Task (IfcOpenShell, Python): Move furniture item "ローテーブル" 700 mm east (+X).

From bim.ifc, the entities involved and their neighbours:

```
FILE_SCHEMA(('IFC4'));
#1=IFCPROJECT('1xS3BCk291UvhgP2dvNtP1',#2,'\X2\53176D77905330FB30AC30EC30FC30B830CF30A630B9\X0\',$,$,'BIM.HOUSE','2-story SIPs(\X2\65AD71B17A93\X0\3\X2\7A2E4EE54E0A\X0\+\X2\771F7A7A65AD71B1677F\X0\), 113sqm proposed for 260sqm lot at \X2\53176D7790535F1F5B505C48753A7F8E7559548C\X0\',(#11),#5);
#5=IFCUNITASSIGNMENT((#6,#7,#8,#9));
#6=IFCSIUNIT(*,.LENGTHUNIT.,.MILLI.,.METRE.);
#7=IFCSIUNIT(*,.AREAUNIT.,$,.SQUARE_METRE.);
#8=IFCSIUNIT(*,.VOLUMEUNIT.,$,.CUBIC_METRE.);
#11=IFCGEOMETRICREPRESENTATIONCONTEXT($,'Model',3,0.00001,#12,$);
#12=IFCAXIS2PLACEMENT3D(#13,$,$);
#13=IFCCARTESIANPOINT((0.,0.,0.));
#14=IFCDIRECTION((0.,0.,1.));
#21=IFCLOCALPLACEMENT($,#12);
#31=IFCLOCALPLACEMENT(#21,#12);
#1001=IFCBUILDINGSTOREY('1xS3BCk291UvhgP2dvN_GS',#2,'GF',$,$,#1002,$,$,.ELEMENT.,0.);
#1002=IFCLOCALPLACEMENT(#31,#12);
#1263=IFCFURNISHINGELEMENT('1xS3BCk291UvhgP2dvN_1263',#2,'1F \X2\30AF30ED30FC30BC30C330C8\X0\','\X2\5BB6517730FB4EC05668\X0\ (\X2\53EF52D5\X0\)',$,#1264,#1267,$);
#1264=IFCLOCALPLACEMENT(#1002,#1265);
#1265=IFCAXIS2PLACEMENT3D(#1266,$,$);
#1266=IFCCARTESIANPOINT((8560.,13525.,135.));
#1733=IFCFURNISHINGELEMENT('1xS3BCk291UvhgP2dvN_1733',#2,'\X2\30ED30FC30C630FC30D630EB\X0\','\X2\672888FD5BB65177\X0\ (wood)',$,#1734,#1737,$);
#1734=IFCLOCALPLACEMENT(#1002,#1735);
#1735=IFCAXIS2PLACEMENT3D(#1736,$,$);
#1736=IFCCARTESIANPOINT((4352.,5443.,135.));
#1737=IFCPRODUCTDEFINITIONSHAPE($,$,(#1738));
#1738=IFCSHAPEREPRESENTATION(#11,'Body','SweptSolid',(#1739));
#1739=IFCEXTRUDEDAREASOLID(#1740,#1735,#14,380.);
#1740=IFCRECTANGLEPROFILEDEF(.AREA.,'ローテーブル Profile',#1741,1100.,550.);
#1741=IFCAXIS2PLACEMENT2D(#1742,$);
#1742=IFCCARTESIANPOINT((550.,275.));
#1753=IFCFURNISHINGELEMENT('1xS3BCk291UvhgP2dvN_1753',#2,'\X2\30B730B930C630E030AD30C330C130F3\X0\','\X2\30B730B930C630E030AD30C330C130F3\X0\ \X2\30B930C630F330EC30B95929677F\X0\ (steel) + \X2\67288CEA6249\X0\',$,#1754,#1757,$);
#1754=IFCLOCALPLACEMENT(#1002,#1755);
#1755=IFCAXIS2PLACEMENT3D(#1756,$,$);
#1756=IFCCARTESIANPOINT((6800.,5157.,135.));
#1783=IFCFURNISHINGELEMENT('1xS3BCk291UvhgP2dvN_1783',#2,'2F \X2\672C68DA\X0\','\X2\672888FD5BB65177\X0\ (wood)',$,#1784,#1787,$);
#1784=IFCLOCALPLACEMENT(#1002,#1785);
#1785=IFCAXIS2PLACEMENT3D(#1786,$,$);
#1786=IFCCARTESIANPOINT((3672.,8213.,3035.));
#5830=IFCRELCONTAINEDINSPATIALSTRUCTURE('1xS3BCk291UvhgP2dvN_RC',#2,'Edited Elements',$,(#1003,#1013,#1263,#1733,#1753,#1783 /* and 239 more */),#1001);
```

```python
import ifcopenshell
import ifcopenshell.api.geometry
import ifcopenshell.util.placement
import ifcopenshell.util.unit

model = ifcopenshell.open("bim.ifc")
unit_scale = ifcopenshell.util.unit.calculate_unit_scale(model)

item = model.by_guid("1xS3BCk291UvhgP2dvN_1733")
matrix = ifcopenshell.util.placement.get_local_placement(item.ObjectPlacement)
matrix[0, 3] += 0.7 / unit_scale
ifcopenshell.api.geometry.edit_object_placement(model, product=item, matrix=matrix, is_si=False)

print(ifcopenshell.util.placement.get_local_placement(item.ObjectPlacement).round(3) + 0.0)

model.write("bim_rev.ifc")
```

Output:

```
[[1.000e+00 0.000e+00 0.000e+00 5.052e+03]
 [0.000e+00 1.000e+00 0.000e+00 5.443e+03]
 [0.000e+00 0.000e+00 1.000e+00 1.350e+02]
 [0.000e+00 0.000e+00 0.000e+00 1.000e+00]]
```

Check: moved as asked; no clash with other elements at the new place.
